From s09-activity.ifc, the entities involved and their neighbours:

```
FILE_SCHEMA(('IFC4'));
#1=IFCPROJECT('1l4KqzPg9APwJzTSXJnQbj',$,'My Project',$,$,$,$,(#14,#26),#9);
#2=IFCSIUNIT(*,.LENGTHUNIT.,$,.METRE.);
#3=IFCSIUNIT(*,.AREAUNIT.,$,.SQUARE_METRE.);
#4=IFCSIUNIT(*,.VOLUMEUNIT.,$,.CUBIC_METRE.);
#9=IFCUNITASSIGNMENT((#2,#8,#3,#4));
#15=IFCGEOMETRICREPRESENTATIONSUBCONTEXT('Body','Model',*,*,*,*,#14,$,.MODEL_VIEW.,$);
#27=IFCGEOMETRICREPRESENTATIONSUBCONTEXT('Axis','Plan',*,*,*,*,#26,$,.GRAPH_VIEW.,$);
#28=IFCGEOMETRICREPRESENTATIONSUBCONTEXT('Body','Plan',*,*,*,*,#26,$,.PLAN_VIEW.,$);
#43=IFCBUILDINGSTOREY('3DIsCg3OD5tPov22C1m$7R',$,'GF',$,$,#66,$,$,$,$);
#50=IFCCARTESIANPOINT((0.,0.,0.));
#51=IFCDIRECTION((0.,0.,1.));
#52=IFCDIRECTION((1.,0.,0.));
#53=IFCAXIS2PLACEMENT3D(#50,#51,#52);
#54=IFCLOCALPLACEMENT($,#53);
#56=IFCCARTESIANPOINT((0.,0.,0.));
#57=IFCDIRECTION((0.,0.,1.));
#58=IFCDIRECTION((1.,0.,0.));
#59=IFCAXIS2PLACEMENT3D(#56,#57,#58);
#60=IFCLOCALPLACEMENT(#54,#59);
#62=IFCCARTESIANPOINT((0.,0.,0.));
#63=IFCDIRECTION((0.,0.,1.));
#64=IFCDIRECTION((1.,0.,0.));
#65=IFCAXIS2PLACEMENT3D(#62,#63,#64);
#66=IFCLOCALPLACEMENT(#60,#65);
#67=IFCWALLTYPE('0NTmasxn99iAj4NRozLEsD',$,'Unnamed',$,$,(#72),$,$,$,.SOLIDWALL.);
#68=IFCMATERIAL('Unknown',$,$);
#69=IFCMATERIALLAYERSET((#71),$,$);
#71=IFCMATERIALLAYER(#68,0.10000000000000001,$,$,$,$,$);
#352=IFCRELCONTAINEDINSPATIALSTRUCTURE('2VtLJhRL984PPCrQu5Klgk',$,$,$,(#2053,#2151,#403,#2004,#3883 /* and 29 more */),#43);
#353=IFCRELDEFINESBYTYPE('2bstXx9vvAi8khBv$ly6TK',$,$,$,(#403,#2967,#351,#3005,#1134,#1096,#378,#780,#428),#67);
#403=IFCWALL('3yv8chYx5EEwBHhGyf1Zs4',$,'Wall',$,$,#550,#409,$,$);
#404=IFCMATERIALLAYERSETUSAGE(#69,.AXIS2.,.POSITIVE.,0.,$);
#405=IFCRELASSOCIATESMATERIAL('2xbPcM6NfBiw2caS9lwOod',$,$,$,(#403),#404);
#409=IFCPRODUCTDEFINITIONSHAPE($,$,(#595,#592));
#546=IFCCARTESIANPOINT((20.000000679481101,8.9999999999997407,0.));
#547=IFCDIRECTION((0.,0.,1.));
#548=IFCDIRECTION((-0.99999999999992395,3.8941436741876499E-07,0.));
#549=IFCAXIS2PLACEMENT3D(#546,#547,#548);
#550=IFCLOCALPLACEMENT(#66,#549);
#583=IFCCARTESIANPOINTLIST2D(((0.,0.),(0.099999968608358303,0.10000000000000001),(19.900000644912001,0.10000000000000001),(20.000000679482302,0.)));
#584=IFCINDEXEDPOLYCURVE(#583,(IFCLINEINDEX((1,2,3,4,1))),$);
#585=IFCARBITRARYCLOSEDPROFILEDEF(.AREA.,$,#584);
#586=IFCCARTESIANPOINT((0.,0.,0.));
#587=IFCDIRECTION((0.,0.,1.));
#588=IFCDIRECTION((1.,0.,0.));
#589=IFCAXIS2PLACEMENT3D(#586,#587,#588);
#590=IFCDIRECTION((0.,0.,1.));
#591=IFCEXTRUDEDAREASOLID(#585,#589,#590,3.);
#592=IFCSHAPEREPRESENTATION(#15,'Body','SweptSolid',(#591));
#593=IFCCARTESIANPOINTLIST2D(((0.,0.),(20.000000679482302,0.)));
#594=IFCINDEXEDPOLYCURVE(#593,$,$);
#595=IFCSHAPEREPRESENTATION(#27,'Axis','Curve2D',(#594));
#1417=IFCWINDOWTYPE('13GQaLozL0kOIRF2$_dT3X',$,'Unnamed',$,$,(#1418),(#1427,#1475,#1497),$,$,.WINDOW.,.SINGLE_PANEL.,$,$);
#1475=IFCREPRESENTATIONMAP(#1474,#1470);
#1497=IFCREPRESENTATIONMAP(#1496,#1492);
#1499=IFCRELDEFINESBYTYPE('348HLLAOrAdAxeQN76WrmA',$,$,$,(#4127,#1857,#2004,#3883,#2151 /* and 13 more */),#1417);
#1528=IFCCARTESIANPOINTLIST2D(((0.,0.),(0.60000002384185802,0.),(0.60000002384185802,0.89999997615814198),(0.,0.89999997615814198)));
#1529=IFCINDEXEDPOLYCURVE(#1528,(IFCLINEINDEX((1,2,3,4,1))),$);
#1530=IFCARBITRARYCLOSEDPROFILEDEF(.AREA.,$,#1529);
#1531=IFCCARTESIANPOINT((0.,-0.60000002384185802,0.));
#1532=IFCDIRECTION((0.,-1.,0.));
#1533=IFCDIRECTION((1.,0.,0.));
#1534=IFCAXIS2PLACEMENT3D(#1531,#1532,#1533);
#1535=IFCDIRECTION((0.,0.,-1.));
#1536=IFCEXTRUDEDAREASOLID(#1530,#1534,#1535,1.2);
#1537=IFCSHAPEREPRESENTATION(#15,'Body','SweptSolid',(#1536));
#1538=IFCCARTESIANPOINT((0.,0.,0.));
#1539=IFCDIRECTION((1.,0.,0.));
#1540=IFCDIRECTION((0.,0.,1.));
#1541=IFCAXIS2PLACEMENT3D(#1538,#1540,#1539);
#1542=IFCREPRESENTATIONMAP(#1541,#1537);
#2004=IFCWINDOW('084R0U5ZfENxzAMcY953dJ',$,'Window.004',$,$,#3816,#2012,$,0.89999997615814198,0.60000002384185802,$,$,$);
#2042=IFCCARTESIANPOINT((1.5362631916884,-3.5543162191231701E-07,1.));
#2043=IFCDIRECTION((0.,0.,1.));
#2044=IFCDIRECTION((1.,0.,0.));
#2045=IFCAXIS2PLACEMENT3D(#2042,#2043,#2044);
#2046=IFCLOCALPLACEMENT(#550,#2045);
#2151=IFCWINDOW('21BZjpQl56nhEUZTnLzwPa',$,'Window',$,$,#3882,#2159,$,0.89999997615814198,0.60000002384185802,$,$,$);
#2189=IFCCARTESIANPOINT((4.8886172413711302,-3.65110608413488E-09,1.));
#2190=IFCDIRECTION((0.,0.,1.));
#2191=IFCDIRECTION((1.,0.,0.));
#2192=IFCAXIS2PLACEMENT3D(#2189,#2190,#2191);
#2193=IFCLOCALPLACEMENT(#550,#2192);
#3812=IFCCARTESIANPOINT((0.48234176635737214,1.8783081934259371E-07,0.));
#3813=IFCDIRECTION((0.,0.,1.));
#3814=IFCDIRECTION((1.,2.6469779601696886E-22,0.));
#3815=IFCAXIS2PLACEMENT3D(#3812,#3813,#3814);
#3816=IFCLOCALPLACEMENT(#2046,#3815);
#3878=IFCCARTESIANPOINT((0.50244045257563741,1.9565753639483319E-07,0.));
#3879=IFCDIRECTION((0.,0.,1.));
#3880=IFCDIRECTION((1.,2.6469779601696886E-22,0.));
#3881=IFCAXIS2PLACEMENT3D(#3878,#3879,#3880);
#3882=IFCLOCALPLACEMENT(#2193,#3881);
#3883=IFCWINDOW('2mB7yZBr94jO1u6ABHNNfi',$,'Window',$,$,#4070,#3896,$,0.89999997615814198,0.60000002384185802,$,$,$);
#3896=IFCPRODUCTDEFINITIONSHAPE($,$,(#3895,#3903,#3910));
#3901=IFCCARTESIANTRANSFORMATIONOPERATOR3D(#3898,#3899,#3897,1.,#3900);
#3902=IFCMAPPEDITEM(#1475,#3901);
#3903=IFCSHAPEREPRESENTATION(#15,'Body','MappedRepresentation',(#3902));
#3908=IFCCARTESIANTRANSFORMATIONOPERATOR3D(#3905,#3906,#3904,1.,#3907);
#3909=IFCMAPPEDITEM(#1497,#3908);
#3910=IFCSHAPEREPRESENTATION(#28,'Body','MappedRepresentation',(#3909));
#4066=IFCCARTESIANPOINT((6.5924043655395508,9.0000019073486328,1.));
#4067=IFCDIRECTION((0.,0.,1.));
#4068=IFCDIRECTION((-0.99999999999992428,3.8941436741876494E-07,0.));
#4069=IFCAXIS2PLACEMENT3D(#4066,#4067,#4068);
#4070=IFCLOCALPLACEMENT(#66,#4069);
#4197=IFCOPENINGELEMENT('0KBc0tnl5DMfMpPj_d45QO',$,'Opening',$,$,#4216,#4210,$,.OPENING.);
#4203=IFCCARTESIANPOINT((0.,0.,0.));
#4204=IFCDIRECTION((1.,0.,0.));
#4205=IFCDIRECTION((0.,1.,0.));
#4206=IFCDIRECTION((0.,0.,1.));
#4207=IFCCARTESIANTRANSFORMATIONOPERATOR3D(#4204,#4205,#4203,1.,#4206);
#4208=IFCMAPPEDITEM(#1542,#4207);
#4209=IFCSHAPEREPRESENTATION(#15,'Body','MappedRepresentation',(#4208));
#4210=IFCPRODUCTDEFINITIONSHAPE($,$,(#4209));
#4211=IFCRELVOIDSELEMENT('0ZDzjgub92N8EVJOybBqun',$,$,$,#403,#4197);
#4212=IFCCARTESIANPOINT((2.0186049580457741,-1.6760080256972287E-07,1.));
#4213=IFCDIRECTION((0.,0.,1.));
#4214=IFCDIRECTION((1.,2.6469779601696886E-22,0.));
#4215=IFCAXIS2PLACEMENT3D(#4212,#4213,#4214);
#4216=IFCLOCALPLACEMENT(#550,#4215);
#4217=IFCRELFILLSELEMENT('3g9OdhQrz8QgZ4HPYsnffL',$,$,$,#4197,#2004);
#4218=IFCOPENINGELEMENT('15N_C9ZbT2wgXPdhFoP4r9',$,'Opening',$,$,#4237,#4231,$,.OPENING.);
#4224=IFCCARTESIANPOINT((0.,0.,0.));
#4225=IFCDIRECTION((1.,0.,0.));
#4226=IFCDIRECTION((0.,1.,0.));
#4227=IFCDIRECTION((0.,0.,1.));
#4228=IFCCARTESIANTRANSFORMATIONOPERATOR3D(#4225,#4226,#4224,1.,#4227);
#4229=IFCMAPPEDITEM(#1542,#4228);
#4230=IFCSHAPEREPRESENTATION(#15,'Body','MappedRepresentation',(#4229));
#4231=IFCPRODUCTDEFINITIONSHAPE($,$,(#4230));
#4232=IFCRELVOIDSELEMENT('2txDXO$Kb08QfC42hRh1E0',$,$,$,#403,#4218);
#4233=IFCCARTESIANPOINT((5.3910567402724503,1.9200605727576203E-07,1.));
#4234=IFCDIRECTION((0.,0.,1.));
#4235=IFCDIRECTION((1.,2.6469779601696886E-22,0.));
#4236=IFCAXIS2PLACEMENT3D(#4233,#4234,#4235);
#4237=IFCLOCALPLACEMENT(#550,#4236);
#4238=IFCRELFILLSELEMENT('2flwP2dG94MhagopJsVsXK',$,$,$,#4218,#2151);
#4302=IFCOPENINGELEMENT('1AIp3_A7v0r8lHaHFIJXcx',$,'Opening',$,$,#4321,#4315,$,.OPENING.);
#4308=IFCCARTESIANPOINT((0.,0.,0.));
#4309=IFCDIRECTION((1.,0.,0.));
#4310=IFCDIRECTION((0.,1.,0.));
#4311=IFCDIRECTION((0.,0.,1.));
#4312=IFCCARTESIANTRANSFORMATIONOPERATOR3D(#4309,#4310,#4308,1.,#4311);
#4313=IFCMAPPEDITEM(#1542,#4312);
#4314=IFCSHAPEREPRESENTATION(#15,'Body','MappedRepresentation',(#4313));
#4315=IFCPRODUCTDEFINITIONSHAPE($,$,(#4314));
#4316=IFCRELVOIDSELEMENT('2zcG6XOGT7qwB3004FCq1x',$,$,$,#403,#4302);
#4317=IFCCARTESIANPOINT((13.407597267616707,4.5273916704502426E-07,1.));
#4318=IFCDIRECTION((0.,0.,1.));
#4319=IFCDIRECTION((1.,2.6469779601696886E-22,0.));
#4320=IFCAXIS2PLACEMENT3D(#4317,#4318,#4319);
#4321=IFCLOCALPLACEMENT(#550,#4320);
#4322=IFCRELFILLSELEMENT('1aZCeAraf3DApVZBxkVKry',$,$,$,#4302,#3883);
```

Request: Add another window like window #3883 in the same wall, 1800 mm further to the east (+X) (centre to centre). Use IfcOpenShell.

```python
import ifcopenshell
import ifcopenshell.api.feature
import ifcopenshell.api.geometry
import ifcopenshell.api.root
import ifcopenshell.geom
import ifcopenshell.util.element
import ifcopenshell.util.placement
import ifcopenshell.util.shape

model = ifcopenshell.open("s09-activity.ifc")
settings = ifcopenshell.geom.settings()


def volume(element):
    """Net volume in cubic metres, openings subtracted."""
    shape = ifcopenshell.geom.create_shape(settings, element)
    return ifcopenshell.util.shape.get_volume(shape.geometry)


window = model.by_guid("2mB7yZBr94jO1u6ABHNNfi")
opening = window.FillsVoids[0].RelatingOpeningElement
wall = opening.VoidsElements[0].RelatingBuildingElement
before = volume(wall)
shift = ifcopenshell.util.placement.get_local_placement(wall.ObjectPlacement)[:3, 0] * -1.8

# copy_class copies the void relationship, type, container and properties, but no geometry.
new_opening = ifcopenshell.api.root.copy_class(model, product=opening)
new_opening.Representation = ifcopenshell.util.element.copy_deep(
    model, opening.Representation, exclude=["IfcGeometricRepresentationContext", "IfcRepresentationMap"]
)
new_window = ifcopenshell.api.root.copy_class(model, product=window)
new_window.Representation = ifcopenshell.util.element.copy_deep(
    model, window.Representation, exclude=["IfcGeometricRepresentationContext", "IfcRepresentationMap"]
)
ifcopenshell.api.feature.add_filling(model, opening=new_opening, element=new_window)

for old, new in ((opening, new_opening), (window, new_window)):
    matrix = ifcopenshell.util.placement.get_local_placement(old.ObjectPlacement)
    matrix[:3, 3] += shift
    ifcopenshell.api.geometry.edit_object_placement(model, product=new, matrix=matrix, is_si=False)

after = volume(wall)

print(f"wall volume {before:.3f} -> {after:.3f} m3")

model.write("s09-activity_updated.ifc")
```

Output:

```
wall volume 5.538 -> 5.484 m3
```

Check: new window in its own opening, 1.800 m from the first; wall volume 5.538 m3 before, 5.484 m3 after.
